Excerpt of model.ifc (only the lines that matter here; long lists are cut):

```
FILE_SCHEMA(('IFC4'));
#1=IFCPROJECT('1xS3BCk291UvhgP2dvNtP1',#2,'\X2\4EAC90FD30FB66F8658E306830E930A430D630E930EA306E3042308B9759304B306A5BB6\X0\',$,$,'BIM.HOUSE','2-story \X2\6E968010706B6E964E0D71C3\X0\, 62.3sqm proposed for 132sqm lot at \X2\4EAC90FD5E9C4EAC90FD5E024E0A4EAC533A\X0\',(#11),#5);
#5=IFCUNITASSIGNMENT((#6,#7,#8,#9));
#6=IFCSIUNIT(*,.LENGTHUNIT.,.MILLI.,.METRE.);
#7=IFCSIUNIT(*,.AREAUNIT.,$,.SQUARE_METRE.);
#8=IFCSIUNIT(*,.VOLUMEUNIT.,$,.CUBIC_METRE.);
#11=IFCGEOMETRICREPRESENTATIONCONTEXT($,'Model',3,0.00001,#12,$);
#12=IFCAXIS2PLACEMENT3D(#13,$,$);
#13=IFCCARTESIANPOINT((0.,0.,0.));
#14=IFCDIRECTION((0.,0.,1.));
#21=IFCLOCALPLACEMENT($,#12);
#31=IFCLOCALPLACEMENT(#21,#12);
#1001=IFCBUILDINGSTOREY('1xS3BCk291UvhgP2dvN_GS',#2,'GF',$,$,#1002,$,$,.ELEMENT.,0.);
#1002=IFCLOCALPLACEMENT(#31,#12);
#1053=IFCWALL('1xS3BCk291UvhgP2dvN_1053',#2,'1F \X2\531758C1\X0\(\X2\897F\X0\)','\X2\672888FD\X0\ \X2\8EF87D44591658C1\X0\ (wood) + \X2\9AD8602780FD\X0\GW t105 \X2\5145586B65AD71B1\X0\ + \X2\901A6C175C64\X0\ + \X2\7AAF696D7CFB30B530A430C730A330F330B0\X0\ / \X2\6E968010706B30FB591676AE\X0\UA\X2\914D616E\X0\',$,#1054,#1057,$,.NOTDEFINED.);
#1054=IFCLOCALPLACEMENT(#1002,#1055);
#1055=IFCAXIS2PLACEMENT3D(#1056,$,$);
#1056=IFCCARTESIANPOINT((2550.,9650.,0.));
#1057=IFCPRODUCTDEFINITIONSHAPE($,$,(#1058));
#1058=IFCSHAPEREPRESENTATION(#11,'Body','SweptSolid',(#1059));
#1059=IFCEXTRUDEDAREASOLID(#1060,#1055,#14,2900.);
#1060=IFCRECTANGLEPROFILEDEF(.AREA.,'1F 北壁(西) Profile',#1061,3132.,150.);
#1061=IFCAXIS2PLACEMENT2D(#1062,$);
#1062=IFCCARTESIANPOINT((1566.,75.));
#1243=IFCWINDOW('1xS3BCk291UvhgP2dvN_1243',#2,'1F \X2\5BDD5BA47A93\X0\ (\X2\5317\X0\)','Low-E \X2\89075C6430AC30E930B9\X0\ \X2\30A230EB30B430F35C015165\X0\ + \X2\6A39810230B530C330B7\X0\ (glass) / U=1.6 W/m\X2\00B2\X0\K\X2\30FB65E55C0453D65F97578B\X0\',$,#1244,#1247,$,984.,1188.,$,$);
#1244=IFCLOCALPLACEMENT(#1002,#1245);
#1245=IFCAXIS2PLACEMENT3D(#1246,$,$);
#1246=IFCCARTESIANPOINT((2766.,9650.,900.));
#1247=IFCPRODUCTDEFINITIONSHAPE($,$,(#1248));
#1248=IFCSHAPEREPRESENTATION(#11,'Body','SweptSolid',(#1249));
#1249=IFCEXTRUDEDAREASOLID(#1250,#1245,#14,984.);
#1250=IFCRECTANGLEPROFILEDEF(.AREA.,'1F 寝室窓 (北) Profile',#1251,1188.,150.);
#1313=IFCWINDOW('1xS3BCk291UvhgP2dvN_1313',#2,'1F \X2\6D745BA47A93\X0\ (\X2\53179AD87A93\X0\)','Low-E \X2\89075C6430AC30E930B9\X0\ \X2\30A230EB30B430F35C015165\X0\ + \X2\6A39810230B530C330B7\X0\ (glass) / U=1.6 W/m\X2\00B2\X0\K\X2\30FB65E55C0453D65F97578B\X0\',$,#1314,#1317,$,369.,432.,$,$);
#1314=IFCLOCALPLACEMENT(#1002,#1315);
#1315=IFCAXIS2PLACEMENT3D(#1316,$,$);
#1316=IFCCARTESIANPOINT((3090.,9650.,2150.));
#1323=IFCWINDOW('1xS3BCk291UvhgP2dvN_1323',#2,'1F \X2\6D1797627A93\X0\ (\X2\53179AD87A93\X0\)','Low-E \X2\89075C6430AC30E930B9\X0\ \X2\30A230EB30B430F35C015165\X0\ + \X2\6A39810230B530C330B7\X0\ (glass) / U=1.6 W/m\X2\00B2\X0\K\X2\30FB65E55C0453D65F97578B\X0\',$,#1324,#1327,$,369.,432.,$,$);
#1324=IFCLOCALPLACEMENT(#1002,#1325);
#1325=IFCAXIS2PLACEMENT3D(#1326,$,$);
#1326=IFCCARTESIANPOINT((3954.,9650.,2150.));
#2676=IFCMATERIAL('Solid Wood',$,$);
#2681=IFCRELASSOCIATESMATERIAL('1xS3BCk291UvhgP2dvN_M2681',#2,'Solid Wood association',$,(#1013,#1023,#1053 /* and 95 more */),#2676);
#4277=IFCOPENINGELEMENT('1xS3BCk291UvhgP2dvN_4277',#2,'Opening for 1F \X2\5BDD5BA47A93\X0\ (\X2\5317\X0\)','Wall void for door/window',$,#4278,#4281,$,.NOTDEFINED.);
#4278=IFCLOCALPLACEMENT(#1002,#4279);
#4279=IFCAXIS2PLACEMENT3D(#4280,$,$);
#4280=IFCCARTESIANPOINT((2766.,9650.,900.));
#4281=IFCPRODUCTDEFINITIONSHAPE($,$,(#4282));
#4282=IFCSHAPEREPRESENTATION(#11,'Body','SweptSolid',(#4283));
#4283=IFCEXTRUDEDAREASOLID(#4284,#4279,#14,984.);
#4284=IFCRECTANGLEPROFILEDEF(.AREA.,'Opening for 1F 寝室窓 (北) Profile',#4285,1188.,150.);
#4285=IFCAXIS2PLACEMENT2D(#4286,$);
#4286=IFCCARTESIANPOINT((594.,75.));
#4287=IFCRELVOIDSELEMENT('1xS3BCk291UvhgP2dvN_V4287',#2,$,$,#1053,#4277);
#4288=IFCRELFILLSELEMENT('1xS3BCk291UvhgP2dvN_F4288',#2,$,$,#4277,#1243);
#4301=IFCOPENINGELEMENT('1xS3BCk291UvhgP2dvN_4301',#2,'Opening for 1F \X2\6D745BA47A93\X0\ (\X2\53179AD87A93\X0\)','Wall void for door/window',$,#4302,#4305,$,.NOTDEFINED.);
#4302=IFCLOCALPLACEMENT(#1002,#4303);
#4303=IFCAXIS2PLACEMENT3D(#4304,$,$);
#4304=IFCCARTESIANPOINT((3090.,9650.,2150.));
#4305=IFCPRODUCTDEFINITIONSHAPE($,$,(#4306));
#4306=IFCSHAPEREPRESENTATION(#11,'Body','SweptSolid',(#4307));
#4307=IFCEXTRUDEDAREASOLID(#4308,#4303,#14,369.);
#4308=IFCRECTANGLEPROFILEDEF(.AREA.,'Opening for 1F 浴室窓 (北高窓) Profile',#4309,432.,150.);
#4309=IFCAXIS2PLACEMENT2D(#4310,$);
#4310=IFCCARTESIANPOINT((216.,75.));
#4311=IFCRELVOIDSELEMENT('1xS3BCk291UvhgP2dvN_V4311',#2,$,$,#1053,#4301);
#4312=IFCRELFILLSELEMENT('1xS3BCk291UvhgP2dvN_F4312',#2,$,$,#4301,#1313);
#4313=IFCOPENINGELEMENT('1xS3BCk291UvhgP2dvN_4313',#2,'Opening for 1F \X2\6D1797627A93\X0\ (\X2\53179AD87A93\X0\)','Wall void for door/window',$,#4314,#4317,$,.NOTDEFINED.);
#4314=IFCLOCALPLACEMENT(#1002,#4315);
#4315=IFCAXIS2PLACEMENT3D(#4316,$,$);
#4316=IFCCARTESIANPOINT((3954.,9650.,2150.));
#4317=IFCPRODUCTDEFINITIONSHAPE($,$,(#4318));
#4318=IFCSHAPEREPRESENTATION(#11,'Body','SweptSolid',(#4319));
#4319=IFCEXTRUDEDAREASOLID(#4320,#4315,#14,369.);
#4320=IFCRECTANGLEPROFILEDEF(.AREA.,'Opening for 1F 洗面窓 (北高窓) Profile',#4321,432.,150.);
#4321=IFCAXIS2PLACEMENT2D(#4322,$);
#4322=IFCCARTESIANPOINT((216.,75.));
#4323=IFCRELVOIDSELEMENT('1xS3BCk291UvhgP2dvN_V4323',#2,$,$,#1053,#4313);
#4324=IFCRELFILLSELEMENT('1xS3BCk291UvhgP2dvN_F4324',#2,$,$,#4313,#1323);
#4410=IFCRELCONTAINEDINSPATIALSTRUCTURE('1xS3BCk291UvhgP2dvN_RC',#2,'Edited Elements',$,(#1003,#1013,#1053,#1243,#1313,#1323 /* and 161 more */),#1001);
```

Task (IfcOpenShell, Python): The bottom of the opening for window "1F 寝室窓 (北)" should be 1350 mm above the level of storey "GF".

```python
import numpy as np
import ifcopenshell
import ifcopenshell.api.geometry
import ifcopenshell.geom
import ifcopenshell.util.element
import ifcopenshell.util.placement
import ifcopenshell.util.shape
import ifcopenshell.util.unit

model = ifcopenshell.open("model.ifc")
unit_scale = ifcopenshell.util.unit.calculate_unit_scale(model)

window = model.by_guid("1xS3BCk291UvhgP2dvN_1243")
opening = window.FillsVoids[0].RelatingOpeningElement
storey = ifcopenshell.util.element.get_container(window, ifc_class="IfcBuildingStorey")
level = ifcopenshell.util.placement.get_local_placement(storey.ObjectPlacement)[2, 3]

# The opening's origin need not be at the sill, so measure its lowest point.
shape = ifcopenshell.geom.create_shape(ifcopenshell.geom.settings(), opening)
bottom = ifcopenshell.util.shape.get_shape_bottom_elevation(shape, shape.geometry) / unit_scale
dz = level + 1.35 / unit_scale - bottom

shift = np.array([0.0, 0.0, dz])
# The window is not placed relative to its opening, so move both.
for product in (opening, window):
    matrix = ifcopenshell.util.placement.get_local_placement(product.ObjectPlacement)
    matrix[:3, 3] += shift
    ifcopenshell.api.geometry.edit_object_placement(model, product=product, matrix=matrix, is_si=False)

print(f"moved by {dz * unit_scale:+.3f} m")

model.write("model_rev.ifc")
```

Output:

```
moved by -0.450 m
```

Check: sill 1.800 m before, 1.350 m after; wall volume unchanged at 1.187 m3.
